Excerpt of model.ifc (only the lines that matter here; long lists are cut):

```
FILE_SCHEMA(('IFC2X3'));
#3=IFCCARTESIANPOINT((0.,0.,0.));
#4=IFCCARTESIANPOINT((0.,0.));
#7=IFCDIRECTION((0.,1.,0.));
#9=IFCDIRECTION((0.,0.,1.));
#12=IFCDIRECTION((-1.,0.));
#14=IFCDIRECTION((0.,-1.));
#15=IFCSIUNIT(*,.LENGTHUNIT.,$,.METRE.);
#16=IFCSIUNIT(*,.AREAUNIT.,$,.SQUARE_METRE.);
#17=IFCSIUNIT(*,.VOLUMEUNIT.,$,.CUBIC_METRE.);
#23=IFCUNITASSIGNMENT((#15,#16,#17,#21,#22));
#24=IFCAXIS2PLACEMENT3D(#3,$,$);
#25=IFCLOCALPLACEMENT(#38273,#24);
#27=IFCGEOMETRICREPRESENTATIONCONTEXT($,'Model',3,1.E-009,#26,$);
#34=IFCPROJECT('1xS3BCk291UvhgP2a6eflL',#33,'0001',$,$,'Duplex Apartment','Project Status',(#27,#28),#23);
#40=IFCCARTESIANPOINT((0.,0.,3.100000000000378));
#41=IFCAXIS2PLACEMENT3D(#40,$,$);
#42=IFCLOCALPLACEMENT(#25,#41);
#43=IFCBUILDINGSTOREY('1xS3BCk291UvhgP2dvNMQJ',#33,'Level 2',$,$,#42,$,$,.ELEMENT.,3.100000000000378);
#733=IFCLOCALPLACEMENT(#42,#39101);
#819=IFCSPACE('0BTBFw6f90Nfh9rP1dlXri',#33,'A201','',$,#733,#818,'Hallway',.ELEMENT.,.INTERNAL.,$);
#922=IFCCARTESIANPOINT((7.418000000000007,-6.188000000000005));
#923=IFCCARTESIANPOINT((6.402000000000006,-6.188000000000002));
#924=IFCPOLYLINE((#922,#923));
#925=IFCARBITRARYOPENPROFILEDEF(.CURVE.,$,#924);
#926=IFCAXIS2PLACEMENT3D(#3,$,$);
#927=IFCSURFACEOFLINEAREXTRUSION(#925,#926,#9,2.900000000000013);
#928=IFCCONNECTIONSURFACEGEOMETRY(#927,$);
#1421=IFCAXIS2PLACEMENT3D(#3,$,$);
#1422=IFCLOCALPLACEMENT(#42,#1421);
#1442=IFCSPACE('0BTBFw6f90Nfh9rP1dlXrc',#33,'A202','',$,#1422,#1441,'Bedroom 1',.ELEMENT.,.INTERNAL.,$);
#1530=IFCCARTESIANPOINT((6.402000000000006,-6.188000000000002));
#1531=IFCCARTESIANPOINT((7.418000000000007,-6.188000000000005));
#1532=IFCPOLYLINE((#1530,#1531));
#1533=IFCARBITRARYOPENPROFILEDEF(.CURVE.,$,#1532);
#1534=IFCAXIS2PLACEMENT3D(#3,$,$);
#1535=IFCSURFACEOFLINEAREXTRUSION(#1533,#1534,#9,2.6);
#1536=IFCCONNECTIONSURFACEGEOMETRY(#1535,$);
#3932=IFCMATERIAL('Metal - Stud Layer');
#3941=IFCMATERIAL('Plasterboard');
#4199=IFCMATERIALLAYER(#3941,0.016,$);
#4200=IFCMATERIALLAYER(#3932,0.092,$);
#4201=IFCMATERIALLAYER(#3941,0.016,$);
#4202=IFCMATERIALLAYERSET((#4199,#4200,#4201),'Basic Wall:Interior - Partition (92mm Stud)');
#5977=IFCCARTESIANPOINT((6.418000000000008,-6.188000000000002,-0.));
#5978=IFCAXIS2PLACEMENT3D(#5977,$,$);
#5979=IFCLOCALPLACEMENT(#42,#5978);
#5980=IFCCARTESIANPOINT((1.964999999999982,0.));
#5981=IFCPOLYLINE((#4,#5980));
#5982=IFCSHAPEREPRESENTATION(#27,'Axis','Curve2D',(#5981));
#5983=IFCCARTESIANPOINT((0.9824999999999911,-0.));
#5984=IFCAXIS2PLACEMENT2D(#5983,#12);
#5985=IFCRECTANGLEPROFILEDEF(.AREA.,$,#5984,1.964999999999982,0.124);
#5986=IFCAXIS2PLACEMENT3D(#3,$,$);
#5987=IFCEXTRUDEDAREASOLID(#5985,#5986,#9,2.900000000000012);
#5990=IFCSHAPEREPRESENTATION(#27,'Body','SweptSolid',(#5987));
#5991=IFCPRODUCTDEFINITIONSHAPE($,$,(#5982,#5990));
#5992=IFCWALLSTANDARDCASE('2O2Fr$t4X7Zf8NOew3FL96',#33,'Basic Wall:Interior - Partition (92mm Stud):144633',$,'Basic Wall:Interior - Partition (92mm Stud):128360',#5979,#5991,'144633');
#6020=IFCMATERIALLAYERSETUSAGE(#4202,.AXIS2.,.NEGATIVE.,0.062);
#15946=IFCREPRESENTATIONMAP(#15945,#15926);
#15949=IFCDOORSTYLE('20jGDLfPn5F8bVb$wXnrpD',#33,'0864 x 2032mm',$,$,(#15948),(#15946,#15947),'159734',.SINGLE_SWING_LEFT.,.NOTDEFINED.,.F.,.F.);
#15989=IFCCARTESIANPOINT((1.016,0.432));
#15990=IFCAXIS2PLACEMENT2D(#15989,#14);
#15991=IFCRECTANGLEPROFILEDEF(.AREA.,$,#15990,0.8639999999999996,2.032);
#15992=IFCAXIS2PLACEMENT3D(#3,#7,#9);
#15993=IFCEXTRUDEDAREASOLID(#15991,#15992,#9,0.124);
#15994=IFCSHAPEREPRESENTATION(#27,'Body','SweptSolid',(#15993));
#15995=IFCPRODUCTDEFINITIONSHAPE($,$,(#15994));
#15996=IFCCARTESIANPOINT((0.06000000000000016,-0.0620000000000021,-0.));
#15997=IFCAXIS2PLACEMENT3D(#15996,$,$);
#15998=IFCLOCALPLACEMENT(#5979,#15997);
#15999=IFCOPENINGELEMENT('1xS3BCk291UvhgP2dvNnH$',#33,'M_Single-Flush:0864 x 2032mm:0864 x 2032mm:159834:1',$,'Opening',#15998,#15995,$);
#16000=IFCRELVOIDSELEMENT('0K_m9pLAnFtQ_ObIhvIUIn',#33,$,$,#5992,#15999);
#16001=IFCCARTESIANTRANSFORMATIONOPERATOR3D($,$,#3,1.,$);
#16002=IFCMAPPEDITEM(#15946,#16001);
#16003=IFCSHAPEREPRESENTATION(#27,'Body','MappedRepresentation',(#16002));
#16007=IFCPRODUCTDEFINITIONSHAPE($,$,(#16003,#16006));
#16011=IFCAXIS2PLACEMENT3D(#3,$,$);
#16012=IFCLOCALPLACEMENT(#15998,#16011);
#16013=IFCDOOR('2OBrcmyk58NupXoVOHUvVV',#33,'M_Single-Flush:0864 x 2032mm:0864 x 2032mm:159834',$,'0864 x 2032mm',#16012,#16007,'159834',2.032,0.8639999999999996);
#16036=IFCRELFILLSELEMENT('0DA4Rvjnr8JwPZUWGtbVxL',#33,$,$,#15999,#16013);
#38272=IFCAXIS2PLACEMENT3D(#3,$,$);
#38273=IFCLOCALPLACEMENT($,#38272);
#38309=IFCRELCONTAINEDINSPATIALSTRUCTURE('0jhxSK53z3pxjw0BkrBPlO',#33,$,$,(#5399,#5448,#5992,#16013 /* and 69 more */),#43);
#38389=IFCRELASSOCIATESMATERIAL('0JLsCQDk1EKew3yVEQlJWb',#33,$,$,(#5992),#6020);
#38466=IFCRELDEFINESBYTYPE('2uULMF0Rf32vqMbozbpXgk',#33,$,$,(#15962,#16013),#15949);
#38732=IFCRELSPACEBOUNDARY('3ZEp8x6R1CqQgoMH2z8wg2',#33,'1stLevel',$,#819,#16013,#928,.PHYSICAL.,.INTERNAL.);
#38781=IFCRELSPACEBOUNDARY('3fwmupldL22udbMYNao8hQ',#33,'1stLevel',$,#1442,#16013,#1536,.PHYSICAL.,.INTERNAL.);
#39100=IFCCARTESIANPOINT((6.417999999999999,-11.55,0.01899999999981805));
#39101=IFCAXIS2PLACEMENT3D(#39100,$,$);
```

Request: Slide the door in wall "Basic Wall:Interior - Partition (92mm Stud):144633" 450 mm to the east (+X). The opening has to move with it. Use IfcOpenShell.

```python
import numpy as np
import ifcopenshell
import ifcopenshell.api.geometry
import ifcopenshell.util.placement

model = ifcopenshell.open("model.ifc")

door = model.by_id(16013)
opening = door.FillsVoids[0].RelatingOpeningElement
wall = opening.VoidsElements[0].RelatingBuildingElement

wall_matrix = ifcopenshell.util.placement.get_local_placement(wall.ObjectPlacement)
shift = wall_matrix[:3, 0] * 0.45
before = ifcopenshell.util.placement.get_local_placement(door.ObjectPlacement)[:3, 3].copy()

# The door is placed relative to its opening, so it follows when the opening moves.
matrix = ifcopenshell.util.placement.get_local_placement(opening.ObjectPlacement)
matrix[:3, 3] += shift
ifcopenshell.api.geometry.edit_object_placement(
    model, product=opening, matrix=matrix, is_si=False, should_transform_children=True
)

# Space boundary surfaces are stored in each space's coordinates; move them too.
for rel in door.ProvidesBoundaries:
    if not rel.ConnectionGeometry:
        continue
    surface = rel.ConnectionGeometry.SurfaceOnRelatingElement
    space_matrix = ifcopenshell.util.placement.get_local_placement(rel.RelatingSpace.ObjectPlacement)
    point = np.array(surface.Position.Location.Coordinates) + space_matrix[:3, :3].T @ shift
    surface.Position = model.createIfcAxis2Placement3D(
        model.createIfcCartesianPoint(point.tolist()), surface.Position.Axis, surface.Position.RefDirection
    )

after = ifcopenshell.util.placement.get_local_placement(door.ObjectPlacement)[:3, 3]
print("door moved by", (after - before).round(3) + 0.0)

model.write("model_updated.ifc")
```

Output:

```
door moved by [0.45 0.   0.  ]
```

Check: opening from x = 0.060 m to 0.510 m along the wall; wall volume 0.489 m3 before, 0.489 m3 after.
